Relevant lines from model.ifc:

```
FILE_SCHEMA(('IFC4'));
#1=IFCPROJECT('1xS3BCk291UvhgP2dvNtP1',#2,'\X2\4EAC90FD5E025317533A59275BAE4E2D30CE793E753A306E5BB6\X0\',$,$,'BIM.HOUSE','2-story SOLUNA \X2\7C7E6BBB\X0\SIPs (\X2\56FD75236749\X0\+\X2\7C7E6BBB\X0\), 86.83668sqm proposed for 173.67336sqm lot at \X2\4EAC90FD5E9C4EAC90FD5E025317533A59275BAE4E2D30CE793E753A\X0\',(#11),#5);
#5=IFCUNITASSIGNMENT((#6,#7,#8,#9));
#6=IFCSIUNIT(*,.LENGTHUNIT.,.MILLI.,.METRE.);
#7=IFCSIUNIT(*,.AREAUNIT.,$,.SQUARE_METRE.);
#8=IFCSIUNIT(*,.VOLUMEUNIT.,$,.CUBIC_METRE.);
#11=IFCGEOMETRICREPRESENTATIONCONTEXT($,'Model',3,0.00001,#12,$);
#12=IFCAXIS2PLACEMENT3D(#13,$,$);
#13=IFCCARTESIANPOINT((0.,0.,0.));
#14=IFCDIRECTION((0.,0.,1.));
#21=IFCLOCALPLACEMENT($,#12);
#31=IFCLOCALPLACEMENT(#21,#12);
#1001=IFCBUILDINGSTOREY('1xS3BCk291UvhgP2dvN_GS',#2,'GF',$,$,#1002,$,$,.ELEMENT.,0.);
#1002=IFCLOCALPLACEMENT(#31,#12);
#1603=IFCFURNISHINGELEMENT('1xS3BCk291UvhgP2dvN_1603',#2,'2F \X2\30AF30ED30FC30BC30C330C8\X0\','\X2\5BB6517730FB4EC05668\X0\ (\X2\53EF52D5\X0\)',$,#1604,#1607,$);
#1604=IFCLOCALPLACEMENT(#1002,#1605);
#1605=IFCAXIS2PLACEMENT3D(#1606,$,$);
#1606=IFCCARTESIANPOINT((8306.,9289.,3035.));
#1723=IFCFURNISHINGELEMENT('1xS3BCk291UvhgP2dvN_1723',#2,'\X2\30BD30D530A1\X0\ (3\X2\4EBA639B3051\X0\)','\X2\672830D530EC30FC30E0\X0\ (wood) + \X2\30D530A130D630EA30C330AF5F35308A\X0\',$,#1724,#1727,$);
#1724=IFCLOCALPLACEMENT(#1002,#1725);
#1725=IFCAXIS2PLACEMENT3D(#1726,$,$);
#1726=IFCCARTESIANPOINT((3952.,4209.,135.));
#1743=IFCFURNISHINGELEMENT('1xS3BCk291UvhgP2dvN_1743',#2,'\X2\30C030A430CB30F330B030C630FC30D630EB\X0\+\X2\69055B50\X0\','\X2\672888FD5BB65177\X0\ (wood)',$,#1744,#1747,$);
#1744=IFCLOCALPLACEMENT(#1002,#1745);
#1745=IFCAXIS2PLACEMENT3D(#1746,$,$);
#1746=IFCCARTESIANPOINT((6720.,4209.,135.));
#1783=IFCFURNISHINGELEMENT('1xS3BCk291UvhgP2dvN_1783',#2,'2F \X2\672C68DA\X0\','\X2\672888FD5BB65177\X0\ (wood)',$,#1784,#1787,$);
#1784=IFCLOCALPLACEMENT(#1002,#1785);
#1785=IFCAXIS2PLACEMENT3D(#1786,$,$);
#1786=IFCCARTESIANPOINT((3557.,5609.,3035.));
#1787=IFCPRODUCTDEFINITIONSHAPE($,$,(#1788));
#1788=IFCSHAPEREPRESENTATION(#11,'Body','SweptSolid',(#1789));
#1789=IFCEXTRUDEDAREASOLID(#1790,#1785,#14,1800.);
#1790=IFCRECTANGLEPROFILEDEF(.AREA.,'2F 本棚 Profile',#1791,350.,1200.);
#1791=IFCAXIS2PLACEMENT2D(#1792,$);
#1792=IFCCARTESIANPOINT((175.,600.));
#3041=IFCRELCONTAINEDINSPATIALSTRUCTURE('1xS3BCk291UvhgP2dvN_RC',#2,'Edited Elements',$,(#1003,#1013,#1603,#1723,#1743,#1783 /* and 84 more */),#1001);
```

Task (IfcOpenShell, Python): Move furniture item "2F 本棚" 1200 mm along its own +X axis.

```python
import ifcopenshell
import ifcopenshell.api.geometry
import ifcopenshell.util.placement
import ifcopenshell.util.unit

model = ifcopenshell.open("model.ifc")
unit_scale = ifcopenshell.util.unit.calculate_unit_scale(model)

item = model.by_guid("1xS3BCk291UvhgP2dvN_1783")
matrix = ifcopenshell.util.placement.get_local_placement(item.ObjectPlacement)
matrix[:3, 3] += matrix[:3, 0] * 1.2 / unit_scale
ifcopenshell.api.geometry.edit_object_placement(model, product=item, matrix=matrix, is_si=False)

print(ifcopenshell.util.placement.get_local_placement(item.ObjectPlacement).round(3) + 0.0)

model.write("model_v2.ifc")
```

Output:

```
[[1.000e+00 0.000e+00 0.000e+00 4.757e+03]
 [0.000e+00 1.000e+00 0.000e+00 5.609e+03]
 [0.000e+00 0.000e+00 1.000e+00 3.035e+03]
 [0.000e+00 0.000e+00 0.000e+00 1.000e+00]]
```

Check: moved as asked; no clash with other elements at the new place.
